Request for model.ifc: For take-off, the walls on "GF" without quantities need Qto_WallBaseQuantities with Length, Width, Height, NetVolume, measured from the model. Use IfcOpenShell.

First a look at what the model holds.

```python
import ifcopenshell
import ifcopenshell.util.element
import ifcopenshell.util.unit

model = ifcopenshell.open("model.ifc")
print(model.schema)
for unit_type in ("LENGTHUNIT", "AREAUNIT", "VOLUMEUNIT"):
    print(unit_type, ifcopenshell.util.unit.calculate_unit_scale(model, unit_type))
storey = next(s for s in model.by_type("IfcBuildingStorey") if s.Name == "GF")
walls = [e for e in ifcopenshell.util.element.get_decomposition(storey) if e.is_a("IfcWall")]
for e in sorted(walls, key=lambda e: e.id()):
    print(e.id(), e.is_a(), e.Name, list(ifcopenshell.util.element.get_psets(e, qtos_only=True)), sep=" | ")
```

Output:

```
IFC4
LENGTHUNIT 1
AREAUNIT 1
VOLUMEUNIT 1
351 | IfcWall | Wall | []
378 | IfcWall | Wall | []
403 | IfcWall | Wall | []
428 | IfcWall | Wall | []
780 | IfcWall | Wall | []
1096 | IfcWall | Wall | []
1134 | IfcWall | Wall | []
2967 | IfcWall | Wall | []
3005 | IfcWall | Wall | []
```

```python
import ifcopenshell
import ifcopenshell.api.pset
import ifcopenshell.geom
import ifcopenshell.util.element
import ifcopenshell.util.shape
import ifcopenshell.util.unit

model = ifcopenshell.open("model.ifc")
unit_scale = ifcopenshell.util.unit.calculate_unit_scale(model)
volume_scale = ifcopenshell.util.unit.calculate_unit_scale(model, "VOLUMEUNIT")
settings = ifcopenshell.geom.settings()

storey = next(s for s in model.by_type("IfcBuildingStorey") if s.Name == "GF")
walls = [e for e in ifcopenshell.util.element.get_decomposition(storey) if e.is_a("IfcWall")]

for e in sorted(walls, key=lambda e: e.id()):
    if ifcopenshell.util.element.get_psets(e, qtos_only=True, should_inherit=False):
        continue
    # Geometry comes back in metres, in the element's own axes.
    shape = ifcopenshell.geom.create_shape(settings, e)
    values = {
        "Length": ifcopenshell.util.shape.get_x(shape.geometry) / unit_scale,
        "Width": ifcopenshell.util.shape.get_y(shape.geometry) / unit_scale,
        "Height": ifcopenshell.util.shape.get_z(shape.geometry) / unit_scale,
        "NetVolume": ifcopenshell.util.shape.get_volume(shape.geometry) / volume_scale,
    }
    qto = ifcopenshell.api.pset.add_qto(model, product=e, name="Qto_WallBaseQuantities")
    ifcopenshell.api.pset.edit_qto(model, qto=qto, properties=values)
    print(e.id(), {k: round(v, 3) for k, v in values.items()})

model.write("model_rev.ifc")
```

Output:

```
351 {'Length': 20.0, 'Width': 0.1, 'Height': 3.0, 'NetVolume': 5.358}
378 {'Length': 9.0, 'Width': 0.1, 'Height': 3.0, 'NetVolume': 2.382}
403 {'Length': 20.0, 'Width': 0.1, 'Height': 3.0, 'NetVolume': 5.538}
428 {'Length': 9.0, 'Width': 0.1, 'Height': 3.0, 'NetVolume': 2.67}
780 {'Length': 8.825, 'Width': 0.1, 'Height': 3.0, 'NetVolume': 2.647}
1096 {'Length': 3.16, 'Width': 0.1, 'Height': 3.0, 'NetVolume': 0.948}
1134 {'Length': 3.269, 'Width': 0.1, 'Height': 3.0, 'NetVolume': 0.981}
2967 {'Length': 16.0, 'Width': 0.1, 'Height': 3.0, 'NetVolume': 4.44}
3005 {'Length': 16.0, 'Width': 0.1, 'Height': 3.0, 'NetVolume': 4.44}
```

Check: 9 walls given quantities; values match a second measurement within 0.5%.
